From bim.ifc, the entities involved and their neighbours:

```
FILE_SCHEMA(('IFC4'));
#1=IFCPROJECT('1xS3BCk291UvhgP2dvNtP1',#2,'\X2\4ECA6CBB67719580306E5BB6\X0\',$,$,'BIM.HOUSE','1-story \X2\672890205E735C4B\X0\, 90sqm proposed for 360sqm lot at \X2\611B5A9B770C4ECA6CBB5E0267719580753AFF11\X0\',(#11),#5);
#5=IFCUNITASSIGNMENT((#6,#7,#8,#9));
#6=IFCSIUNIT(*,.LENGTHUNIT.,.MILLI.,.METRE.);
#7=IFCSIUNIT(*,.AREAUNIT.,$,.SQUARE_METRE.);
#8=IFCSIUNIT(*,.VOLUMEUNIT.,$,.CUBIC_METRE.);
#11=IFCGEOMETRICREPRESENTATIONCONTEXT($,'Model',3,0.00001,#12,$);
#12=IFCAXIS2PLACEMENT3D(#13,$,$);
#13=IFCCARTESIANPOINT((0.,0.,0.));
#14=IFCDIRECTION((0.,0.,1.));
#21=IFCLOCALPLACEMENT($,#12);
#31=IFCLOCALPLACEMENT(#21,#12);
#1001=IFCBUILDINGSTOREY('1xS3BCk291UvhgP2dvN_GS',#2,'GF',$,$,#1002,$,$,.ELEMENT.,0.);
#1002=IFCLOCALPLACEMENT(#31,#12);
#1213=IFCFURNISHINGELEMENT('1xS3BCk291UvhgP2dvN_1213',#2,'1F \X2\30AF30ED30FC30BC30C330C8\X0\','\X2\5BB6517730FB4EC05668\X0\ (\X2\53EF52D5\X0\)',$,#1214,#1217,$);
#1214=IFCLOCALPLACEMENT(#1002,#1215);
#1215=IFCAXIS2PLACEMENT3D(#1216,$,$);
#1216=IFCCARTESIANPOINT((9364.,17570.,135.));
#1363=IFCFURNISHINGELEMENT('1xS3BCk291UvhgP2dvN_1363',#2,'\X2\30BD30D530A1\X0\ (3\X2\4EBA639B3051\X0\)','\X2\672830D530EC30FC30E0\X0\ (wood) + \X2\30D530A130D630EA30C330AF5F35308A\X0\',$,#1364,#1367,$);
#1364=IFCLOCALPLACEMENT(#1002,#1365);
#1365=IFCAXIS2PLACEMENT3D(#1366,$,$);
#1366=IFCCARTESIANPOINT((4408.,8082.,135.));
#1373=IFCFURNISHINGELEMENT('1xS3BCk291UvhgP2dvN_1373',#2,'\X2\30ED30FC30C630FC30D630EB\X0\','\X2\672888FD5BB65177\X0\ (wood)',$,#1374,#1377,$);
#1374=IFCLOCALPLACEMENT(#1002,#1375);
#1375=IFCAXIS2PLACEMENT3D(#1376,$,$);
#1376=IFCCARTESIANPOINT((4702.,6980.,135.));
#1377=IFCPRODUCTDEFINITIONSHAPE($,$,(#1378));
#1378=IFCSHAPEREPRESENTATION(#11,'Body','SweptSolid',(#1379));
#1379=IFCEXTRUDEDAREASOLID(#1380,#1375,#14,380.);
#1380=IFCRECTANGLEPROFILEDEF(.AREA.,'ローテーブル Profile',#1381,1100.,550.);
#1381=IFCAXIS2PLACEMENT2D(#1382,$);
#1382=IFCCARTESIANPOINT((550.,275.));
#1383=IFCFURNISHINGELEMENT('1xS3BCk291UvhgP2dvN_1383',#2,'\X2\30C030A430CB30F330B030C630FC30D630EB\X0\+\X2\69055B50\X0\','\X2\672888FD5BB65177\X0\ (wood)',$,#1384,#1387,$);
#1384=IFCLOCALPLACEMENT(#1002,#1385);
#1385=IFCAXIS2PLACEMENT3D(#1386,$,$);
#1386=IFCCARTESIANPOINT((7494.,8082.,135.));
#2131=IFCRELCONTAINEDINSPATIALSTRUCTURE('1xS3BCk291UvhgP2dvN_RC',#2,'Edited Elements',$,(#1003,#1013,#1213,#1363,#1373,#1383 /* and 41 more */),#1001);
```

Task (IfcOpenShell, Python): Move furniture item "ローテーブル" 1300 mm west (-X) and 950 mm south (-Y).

```python
import ifcopenshell
import ifcopenshell.api.geometry
import ifcopenshell.util.placement
import ifcopenshell.util.unit

model = ifcopenshell.open("bim.ifc")
unit_scale = ifcopenshell.util.unit.calculate_unit_scale(model)

item = model.by_guid("1xS3BCk291UvhgP2dvN_1373")
matrix = ifcopenshell.util.placement.get_local_placement(item.ObjectPlacement)
matrix[0, 3] -= 1.3 / unit_scale
matrix[1, 3] -= 0.95 / unit_scale
ifcopenshell.api.geometry.edit_object_placement(model, product=item, matrix=matrix, is_si=False)

print(ifcopenshell.util.placement.get_local_placement(item.ObjectPlacement).round(3) + 0.0)

model.write("bim_v2.ifc")
```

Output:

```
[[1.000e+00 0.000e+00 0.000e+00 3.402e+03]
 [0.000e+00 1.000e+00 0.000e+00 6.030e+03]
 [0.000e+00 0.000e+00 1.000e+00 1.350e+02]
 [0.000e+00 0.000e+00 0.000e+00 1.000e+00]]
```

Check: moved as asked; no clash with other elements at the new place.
